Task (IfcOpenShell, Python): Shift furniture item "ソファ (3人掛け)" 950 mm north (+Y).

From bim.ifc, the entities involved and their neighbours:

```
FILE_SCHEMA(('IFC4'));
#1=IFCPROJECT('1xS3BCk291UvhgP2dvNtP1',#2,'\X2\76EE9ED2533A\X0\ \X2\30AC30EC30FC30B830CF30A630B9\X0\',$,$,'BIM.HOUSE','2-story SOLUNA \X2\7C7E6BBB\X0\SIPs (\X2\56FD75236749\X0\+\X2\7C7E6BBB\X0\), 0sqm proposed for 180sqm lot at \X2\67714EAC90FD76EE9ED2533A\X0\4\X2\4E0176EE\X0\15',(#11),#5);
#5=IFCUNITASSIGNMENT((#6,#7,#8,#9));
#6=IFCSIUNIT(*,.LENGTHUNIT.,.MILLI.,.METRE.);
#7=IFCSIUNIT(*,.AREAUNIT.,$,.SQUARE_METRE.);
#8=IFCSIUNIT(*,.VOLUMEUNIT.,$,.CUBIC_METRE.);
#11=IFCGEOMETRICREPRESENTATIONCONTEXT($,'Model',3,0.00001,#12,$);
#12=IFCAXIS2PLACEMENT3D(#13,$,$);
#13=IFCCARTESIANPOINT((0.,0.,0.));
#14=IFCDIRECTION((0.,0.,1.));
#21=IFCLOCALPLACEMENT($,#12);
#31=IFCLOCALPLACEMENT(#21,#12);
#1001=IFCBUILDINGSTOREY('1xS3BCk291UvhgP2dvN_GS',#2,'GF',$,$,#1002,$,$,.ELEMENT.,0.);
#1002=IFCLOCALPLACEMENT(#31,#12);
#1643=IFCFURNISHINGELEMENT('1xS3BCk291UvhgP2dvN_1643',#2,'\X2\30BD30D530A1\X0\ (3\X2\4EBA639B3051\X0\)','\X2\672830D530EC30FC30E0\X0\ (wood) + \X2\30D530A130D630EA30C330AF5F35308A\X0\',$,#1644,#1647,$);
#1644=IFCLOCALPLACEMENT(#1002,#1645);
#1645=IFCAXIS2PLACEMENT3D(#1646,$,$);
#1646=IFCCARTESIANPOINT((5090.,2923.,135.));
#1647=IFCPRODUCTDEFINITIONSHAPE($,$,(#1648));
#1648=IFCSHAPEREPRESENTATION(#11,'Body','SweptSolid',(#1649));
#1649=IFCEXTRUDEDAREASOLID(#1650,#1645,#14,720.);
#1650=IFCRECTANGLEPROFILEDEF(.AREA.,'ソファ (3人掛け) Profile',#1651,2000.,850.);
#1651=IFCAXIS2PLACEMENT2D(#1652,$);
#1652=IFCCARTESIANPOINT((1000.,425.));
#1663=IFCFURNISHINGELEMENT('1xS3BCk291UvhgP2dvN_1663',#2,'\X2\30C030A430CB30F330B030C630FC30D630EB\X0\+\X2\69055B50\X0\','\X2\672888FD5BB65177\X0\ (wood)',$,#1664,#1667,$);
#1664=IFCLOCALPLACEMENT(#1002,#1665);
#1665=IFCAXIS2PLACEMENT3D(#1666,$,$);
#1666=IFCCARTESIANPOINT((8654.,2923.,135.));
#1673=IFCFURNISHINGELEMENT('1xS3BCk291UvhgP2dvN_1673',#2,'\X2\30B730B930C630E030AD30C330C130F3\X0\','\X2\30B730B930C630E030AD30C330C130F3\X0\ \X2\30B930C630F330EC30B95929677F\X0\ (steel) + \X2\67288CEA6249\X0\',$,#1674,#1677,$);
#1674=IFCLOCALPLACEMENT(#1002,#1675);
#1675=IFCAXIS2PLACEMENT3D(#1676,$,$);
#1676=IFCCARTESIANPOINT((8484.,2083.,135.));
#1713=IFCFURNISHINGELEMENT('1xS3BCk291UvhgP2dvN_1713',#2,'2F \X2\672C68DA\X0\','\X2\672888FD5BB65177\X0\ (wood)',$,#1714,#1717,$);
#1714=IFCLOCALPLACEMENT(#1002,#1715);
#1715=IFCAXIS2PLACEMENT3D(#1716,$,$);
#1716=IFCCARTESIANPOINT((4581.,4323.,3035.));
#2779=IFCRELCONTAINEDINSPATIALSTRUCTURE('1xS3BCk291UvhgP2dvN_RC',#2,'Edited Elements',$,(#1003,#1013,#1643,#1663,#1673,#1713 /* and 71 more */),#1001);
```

```python
import ifcopenshell
import ifcopenshell.api.geometry
import ifcopenshell.util.placement

model = ifcopenshell.open("bim.ifc")

item = model.by_guid("1xS3BCk291UvhgP2dvN_1643")
matrix = ifcopenshell.util.placement.get_local_placement(item.ObjectPlacement)
matrix[1, 3] += 950.0
ifcopenshell.api.geometry.edit_object_placement(model, product=item, matrix=matrix, is_si=False)

print(ifcopenshell.util.placement.get_local_placement(item.ObjectPlacement).round(3) + 0.0)

model.write("bim_v2.ifc")
```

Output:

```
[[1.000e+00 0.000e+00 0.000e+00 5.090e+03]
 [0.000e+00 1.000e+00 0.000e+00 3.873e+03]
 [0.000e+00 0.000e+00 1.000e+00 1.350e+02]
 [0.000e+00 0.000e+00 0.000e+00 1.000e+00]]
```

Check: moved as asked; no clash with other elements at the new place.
